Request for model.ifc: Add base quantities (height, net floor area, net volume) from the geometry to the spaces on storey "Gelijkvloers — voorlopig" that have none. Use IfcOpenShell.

First a look at what the model holds.

```python
import ifcopenshell
import ifcopenshell.util.element
import ifcopenshell.util.unit

model = ifcopenshell.open("model.ifc")
print(model.schema)
for unit_type in ("LENGTHUNIT", "AREAUNIT", "VOLUMEUNIT"):
    print(unit_type, ifcopenshell.util.unit.calculate_unit_scale(model, unit_type))
storey = next(s for s in model.by_type("IfcBuildingStorey") if s.Name == "Gelijkvloers — voorlopig")
spaces = [e for e in ifcopenshell.util.element.get_decomposition(storey) if e.is_a("IfcSpace")]
for e in sorted(spaces, key=lambda e: e.id()):
    print(e.id(), e.is_a(), e.Name, list(ifcopenshell.util.element.get_psets(e, qtos_only=True)), sep=" | ")
```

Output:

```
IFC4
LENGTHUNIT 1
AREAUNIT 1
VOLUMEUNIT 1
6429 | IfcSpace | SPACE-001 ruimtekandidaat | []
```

```python
import ifcopenshell
import ifcopenshell.api.pset
import ifcopenshell.geom
import ifcopenshell.util.element
import ifcopenshell.util.shape
import ifcopenshell.util.unit

model = ifcopenshell.open("model.ifc")
unit_scale = ifcopenshell.util.unit.calculate_unit_scale(model)
area_scale = ifcopenshell.util.unit.calculate_unit_scale(model, "AREAUNIT")
volume_scale = ifcopenshell.util.unit.calculate_unit_scale(model, "VOLUMEUNIT")
settings = ifcopenshell.geom.settings()

storey = next(s for s in model.by_type("IfcBuildingStorey") if s.Name == "Gelijkvloers — voorlopig")
spaces = [e for e in ifcopenshell.util.element.get_decomposition(storey) if e.is_a("IfcSpace")]

for e in sorted(spaces, key=lambda e: e.id()):
    if ifcopenshell.util.element.get_psets(e, qtos_only=True, should_inherit=False):
        continue
    # Geometry comes back in metres, in the element's own axes.
    shape = ifcopenshell.geom.create_shape(settings, e)
    values = {
        "Height": ifcopenshell.util.shape.get_z(shape.geometry) / unit_scale,
        "NetFloorArea": ifcopenshell.util.shape.get_footprint_area(shape.geometry) / area_scale,
        "NetVolume": ifcopenshell.util.shape.get_volume(shape.geometry) / volume_scale,
    }
    qto = ifcopenshell.api.pset.add_qto(model, product=e, name="Qto_SpaceBaseQuantities")
    ifcopenshell.api.pset.edit_qto(model, qto=qto, properties=values)
    print(e.id(), {k: round(v, 3) for k, v in values.items()})

model.write("model-out.ifc")
```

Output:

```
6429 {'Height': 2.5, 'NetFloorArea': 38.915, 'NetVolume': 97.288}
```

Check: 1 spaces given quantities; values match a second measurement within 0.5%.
